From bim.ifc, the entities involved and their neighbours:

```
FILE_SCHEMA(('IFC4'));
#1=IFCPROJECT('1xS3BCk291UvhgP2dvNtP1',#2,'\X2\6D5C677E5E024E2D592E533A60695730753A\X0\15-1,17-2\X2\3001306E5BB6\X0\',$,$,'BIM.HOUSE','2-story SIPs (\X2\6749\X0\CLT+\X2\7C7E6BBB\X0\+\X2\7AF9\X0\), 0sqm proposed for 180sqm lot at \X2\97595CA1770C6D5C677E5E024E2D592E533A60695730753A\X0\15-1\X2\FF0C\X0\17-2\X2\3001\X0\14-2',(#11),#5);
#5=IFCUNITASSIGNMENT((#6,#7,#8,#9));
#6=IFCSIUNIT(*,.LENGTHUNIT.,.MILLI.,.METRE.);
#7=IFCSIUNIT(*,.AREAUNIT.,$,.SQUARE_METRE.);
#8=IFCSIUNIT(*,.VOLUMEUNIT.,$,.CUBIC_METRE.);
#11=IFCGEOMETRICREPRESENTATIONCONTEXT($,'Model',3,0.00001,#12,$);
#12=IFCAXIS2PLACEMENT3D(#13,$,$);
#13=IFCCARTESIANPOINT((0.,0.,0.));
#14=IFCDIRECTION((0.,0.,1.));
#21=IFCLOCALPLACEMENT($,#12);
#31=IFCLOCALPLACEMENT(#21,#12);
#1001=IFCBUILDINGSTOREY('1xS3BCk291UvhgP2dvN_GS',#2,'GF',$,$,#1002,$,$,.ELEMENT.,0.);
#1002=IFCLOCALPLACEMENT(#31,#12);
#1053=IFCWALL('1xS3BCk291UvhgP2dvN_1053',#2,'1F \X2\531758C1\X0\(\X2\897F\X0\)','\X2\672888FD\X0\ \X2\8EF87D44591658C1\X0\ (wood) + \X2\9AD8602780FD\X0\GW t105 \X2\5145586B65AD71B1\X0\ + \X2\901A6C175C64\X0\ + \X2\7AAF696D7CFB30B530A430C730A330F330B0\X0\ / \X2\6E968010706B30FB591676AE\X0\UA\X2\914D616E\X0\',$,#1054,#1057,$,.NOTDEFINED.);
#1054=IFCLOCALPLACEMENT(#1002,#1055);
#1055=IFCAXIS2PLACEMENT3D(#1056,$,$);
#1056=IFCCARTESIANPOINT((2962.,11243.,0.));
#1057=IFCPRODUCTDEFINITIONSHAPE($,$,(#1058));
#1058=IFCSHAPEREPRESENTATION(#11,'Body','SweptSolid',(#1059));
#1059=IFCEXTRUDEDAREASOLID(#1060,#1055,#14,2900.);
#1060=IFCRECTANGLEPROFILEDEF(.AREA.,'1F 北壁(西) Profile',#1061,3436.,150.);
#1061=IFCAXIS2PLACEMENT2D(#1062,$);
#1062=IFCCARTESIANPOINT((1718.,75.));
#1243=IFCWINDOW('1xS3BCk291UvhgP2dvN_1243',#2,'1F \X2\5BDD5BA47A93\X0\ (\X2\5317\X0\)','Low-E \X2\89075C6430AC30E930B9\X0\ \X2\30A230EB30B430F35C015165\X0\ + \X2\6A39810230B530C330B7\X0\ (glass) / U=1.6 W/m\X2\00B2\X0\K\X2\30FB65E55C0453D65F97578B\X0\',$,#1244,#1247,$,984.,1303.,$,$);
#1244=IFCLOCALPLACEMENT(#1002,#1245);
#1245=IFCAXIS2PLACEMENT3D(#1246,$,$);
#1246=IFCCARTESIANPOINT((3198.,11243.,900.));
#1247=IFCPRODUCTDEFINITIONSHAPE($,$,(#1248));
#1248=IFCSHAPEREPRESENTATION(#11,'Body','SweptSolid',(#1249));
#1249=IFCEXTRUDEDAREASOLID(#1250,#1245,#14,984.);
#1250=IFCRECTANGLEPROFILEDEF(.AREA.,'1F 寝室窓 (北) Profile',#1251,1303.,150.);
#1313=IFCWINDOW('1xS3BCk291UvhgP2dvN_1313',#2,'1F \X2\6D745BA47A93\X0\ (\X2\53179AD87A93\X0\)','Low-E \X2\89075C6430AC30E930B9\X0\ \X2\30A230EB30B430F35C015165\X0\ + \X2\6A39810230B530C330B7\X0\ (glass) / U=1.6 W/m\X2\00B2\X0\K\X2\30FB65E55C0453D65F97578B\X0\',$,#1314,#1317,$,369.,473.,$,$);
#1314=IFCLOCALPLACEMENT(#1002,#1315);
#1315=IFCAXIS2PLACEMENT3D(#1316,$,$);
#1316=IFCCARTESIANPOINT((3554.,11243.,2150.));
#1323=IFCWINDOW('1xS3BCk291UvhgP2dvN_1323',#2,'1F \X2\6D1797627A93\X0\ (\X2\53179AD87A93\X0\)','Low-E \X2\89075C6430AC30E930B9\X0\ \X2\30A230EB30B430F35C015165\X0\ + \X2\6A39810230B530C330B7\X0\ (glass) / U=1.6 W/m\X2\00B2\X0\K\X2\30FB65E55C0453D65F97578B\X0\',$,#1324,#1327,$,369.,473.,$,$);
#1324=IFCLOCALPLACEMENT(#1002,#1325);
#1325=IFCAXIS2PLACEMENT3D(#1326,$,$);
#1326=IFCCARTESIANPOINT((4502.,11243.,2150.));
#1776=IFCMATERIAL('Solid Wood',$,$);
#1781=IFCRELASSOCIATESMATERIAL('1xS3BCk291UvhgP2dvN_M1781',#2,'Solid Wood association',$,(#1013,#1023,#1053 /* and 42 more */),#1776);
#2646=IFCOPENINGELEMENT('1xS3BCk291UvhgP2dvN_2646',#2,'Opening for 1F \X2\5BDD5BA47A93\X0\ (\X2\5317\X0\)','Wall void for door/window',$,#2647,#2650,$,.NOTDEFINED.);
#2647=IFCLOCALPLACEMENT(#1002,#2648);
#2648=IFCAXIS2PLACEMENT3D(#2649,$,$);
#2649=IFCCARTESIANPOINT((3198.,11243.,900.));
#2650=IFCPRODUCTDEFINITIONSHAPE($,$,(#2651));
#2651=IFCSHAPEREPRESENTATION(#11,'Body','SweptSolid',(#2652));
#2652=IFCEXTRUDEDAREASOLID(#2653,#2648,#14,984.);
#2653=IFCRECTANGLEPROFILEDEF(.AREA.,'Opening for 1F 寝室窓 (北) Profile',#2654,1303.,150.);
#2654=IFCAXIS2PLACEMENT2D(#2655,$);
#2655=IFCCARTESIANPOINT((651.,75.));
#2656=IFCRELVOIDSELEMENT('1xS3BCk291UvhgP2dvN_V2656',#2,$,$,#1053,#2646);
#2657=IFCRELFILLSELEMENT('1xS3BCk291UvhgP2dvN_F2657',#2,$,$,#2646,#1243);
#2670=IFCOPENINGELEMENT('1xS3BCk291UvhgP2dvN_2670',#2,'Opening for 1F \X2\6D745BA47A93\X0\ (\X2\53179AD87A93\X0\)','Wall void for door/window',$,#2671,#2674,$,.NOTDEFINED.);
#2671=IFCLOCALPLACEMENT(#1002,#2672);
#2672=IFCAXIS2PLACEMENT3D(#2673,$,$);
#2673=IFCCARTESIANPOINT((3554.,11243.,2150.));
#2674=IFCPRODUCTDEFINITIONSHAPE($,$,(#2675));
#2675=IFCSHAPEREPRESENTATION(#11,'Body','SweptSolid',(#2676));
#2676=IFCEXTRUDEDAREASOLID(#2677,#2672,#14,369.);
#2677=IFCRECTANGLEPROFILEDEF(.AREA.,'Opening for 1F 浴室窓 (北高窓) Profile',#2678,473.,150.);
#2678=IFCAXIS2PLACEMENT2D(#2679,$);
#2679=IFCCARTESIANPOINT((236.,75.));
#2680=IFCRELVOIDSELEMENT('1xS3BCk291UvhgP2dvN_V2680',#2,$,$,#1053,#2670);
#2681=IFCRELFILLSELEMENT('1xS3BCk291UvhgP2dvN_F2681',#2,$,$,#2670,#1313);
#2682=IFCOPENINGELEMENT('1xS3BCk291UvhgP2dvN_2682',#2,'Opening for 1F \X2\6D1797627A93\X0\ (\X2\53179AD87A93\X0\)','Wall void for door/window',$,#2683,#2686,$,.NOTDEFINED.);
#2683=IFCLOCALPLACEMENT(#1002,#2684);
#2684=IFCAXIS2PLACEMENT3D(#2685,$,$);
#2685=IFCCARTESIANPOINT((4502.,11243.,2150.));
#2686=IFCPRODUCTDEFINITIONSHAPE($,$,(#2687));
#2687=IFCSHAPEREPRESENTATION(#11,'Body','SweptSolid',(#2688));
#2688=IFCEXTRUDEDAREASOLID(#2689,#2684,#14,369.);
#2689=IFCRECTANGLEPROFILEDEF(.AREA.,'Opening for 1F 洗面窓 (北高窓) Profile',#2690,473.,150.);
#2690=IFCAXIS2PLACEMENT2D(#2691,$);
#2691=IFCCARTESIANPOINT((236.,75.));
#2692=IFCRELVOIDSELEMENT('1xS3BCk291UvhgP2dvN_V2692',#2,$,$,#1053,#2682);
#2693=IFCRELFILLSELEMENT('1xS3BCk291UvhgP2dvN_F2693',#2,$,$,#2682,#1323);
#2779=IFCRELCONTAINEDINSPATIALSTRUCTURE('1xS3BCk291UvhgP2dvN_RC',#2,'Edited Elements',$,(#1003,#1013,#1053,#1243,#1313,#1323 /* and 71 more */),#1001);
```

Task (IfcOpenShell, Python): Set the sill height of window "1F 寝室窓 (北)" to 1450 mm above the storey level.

```python
import numpy as np
import ifcopenshell
import ifcopenshell.api.geometry
import ifcopenshell.geom
import ifcopenshell.util.element
import ifcopenshell.util.placement
import ifcopenshell.util.shape
import ifcopenshell.util.unit

model = ifcopenshell.open("bim.ifc")
unit_scale = ifcopenshell.util.unit.calculate_unit_scale(model)

window = model.by_guid("1xS3BCk291UvhgP2dvN_1243")
opening = window.FillsVoids[0].RelatingOpeningElement
storey = ifcopenshell.util.element.get_container(window, ifc_class="IfcBuildingStorey")
level = ifcopenshell.util.placement.get_local_placement(storey.ObjectPlacement)[2, 3]

# The opening's origin need not be at the sill, so measure its lowest point.
shape = ifcopenshell.geom.create_shape(ifcopenshell.geom.settings(), opening)
bottom = ifcopenshell.util.shape.get_shape_bottom_elevation(shape, shape.geometry) / unit_scale
dz = level + 1450.0 - bottom

shift = np.array([0.0, 0.0, dz])
# The window is not placed relative to its opening, so move both.
for product in (opening, window):
    matrix = ifcopenshell.util.placement.get_local_placement(product.ObjectPlacement)
    matrix[:3, 3] += shift
    ifcopenshell.api.geometry.edit_object_placement(model, product=product, matrix=matrix, is_si=False)

print(f"moved by {dz * unit_scale:+.3f} m")

model.write("bim_updated.ifc")
```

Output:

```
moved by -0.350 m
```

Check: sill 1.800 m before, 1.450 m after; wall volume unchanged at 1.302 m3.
